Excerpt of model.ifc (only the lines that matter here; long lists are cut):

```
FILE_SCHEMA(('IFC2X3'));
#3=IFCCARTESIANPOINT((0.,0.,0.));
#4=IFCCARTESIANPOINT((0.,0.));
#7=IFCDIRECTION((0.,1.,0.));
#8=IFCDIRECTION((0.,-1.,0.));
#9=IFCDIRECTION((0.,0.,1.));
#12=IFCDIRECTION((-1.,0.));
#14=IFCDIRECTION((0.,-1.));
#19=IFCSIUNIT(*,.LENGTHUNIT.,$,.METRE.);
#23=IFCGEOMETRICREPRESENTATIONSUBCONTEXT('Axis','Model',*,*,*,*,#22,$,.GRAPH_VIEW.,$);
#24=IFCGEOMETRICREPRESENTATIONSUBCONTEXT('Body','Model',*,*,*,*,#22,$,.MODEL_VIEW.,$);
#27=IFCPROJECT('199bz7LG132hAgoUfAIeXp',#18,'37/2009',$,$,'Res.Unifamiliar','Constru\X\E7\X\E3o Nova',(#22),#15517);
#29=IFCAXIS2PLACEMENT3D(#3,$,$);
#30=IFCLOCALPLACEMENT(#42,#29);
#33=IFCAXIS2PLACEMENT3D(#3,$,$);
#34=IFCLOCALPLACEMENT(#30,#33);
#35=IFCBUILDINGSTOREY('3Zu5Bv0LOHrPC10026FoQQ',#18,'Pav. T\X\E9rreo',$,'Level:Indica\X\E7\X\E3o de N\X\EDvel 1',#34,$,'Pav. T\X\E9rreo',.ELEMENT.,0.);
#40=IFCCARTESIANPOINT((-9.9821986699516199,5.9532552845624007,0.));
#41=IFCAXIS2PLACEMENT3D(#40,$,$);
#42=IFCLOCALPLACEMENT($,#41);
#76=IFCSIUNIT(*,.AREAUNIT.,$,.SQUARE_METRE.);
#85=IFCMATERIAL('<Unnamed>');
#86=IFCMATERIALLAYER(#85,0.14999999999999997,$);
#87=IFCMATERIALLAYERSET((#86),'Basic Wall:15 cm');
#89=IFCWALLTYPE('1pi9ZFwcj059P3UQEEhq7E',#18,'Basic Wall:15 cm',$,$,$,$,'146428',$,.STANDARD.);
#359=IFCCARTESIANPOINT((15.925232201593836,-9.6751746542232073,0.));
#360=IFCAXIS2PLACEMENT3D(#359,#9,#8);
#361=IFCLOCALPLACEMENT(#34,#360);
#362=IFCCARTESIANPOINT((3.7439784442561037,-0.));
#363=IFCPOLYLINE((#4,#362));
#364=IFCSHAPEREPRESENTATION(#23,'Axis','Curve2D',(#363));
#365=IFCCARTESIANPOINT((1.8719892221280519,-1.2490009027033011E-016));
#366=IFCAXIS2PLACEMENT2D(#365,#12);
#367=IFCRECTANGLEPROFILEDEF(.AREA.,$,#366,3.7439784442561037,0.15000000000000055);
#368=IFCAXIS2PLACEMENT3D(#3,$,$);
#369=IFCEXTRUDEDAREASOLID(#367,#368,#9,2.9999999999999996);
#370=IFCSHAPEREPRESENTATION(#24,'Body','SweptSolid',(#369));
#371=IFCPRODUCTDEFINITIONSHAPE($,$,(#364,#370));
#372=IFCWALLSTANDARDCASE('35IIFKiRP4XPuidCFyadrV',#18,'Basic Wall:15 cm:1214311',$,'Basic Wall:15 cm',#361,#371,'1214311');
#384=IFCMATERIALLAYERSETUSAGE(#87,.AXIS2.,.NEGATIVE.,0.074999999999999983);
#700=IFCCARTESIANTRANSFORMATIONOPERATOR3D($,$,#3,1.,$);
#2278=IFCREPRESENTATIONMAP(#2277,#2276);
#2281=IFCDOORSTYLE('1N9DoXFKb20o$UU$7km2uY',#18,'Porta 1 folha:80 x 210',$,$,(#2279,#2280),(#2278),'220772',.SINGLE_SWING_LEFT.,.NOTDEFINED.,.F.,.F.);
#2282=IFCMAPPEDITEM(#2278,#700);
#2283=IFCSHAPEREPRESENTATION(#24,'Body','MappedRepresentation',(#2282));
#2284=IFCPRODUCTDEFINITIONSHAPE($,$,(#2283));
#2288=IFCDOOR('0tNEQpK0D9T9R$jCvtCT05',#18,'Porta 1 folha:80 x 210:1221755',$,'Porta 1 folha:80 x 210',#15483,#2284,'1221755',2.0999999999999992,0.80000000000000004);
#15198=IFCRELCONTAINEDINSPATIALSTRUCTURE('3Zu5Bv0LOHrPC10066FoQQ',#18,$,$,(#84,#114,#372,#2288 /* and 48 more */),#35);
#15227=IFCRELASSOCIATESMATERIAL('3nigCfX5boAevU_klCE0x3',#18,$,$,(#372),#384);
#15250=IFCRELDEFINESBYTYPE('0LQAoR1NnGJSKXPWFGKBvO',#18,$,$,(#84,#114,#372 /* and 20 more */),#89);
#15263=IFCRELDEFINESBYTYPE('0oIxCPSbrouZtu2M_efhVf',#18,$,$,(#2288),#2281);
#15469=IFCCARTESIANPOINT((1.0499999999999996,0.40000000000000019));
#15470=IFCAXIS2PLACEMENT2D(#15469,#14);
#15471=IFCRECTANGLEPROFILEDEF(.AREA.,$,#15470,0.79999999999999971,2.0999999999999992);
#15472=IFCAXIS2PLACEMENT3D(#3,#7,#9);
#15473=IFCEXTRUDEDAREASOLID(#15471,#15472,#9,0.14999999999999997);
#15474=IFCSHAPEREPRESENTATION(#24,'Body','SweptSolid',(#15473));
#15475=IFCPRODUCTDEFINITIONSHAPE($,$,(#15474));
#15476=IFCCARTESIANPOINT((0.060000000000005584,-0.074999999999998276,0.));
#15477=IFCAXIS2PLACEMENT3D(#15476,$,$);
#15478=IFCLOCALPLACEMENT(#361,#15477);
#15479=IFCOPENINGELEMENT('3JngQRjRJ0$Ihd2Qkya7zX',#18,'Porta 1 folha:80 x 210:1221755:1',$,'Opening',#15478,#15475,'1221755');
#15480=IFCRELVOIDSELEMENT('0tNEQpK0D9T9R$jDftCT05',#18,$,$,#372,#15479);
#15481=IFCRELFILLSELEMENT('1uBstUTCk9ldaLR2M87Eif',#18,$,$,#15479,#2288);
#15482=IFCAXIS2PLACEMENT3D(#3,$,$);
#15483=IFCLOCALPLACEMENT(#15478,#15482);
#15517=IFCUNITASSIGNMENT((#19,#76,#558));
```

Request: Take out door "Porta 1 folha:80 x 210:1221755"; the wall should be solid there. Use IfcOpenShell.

```python
import ifcopenshell
import ifcopenshell.api.feature
import ifcopenshell.api.root
import ifcopenshell.geom
import ifcopenshell.util.shape

model = ifcopenshell.open("model.ifc")
settings = ifcopenshell.geom.settings()


def volume(element):
    """Net volume in cubic metres, openings subtracted."""
    shape = ifcopenshell.geom.create_shape(settings, element)
    return ifcopenshell.util.shape.get_volume(shape.geometry)


door = model.by_guid("0tNEQpK0D9T9R$jCvtCT05")
opening = door.FillsVoids[0].RelatingOpeningElement
wall = opening.VoidsElements[0].RelatingBuildingElement
before = volume(wall)

ifcopenshell.api.root.remove_product(model, product=door)
ifcopenshell.api.feature.remove_feature(model, feature=opening)

after = volume(wall)

print(f"wall volume {before:.3f} -> {after:.3f} m3")

model.write("model_updated.ifc")
```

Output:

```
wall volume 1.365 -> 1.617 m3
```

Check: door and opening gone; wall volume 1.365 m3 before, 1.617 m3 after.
